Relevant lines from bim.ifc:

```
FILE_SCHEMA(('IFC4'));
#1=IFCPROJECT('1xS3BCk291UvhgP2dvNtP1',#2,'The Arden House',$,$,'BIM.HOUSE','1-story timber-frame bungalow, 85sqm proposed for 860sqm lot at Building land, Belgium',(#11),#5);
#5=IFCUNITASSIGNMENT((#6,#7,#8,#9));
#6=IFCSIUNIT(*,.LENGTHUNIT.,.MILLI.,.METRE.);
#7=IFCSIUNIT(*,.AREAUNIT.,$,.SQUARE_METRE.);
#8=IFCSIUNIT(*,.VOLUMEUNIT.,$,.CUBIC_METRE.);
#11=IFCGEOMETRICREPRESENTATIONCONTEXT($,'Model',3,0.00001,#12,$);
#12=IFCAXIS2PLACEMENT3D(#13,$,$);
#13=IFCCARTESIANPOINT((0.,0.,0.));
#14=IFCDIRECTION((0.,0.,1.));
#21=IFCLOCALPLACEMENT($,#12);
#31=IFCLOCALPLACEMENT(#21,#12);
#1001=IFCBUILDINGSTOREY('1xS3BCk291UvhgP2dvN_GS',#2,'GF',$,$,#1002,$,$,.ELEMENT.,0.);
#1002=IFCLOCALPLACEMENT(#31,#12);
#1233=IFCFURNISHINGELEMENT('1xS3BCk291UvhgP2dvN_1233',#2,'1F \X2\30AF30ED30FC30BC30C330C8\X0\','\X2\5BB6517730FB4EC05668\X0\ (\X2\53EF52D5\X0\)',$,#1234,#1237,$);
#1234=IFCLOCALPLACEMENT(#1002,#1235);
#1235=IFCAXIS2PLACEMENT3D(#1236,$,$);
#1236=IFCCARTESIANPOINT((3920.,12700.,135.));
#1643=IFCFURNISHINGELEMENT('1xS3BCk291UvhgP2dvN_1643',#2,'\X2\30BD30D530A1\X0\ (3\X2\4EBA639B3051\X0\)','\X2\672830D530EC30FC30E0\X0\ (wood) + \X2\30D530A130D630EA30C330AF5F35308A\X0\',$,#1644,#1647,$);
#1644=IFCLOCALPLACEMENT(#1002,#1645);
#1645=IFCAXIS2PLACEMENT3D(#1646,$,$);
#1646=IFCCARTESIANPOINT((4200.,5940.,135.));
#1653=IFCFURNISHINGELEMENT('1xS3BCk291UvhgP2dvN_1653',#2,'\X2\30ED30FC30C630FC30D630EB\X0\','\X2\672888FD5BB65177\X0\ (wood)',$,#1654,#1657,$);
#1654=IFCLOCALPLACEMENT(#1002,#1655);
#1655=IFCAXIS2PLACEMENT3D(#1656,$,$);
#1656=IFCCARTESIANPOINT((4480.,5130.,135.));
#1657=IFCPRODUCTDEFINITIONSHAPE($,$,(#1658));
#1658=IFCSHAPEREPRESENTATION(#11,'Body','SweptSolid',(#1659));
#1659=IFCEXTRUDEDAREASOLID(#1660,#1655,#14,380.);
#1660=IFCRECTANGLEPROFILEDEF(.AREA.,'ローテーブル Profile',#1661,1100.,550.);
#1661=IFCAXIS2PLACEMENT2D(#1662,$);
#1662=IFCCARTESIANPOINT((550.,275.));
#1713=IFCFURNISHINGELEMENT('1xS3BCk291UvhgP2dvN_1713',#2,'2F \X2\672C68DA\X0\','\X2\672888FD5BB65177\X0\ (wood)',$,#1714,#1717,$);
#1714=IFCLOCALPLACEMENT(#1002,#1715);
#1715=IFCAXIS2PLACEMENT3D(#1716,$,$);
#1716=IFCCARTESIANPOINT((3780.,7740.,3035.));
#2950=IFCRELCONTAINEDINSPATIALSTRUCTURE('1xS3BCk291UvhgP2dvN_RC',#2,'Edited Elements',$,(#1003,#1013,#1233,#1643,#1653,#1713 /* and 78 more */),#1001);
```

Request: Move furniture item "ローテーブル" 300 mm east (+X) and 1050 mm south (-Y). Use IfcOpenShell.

```python
import ifcopenshell
import ifcopenshell.api.geometry
import ifcopenshell.util.placement
import ifcopenshell.util.unit

model = ifcopenshell.open("bim.ifc")
unit_scale = ifcopenshell.util.unit.calculate_unit_scale(model)

item = model.by_guid("1xS3BCk291UvhgP2dvN_1653")
matrix = ifcopenshell.util.placement.get_local_placement(item.ObjectPlacement)
matrix[0, 3] += 0.3 / unit_scale
matrix[1, 3] -= 1.05 / unit_scale
ifcopenshell.api.geometry.edit_object_placement(model, product=item, matrix=matrix, is_si=False)

print(ifcopenshell.util.placement.get_local_placement(item.ObjectPlacement).round(3) + 0.0)

model.write("bim_rev.ifc")
```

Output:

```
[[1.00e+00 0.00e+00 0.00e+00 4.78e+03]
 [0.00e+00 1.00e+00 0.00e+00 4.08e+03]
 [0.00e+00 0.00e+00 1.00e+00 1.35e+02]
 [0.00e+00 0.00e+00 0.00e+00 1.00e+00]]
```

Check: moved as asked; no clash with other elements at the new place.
